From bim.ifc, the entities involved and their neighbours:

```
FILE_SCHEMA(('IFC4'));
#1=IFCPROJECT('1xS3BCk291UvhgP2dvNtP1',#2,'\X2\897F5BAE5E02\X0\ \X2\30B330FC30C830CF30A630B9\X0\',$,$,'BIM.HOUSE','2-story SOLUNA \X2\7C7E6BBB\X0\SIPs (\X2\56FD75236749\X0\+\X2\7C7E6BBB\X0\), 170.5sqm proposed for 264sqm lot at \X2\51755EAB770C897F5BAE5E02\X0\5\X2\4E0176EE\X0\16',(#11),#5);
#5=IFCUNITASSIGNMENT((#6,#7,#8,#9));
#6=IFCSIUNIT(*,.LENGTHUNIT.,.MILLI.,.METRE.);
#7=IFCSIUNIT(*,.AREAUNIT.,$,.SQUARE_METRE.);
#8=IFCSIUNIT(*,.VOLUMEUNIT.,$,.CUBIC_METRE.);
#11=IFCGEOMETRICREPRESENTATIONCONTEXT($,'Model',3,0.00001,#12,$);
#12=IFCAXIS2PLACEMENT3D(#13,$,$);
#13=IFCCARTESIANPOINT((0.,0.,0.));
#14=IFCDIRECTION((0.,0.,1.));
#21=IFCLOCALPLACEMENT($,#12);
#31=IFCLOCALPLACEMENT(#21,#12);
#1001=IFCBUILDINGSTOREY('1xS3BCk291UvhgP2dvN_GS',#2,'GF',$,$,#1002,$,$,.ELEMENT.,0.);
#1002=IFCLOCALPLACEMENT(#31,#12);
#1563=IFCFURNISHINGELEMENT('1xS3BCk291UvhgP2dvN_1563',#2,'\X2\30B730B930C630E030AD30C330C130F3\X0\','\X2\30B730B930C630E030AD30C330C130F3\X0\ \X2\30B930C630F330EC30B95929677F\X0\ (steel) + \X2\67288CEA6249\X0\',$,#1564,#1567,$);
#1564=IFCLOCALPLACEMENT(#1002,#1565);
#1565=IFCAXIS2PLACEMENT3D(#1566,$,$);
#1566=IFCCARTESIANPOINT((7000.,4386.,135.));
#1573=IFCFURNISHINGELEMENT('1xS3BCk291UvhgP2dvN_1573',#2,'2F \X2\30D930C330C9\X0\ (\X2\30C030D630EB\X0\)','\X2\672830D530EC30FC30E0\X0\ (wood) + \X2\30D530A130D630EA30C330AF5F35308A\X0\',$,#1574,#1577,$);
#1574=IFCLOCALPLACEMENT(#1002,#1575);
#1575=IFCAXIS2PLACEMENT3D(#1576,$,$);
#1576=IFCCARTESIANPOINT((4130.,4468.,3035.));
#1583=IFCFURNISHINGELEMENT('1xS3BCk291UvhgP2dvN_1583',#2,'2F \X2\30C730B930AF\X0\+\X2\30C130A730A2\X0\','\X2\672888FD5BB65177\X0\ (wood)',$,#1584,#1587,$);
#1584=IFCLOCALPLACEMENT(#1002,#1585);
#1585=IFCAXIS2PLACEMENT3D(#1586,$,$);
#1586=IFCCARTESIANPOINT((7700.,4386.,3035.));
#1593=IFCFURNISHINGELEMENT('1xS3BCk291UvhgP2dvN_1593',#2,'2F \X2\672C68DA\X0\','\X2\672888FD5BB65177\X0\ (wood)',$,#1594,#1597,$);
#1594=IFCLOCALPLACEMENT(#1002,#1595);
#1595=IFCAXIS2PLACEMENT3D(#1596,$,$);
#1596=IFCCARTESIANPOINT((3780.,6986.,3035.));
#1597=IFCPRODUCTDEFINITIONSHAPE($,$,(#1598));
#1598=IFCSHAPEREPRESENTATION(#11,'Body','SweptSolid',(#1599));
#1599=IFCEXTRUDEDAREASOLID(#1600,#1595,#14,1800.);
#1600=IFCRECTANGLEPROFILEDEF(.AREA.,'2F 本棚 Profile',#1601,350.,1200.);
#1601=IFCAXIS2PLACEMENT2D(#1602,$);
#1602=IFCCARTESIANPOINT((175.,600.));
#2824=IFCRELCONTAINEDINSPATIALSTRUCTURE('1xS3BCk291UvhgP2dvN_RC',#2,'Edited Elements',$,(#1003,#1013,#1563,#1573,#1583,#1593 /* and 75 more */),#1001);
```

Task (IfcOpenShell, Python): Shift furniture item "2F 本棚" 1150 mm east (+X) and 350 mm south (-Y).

```python
import ifcopenshell
import ifcopenshell.api.geometry
import ifcopenshell.util.placement
import ifcopenshell.util.unit

model = ifcopenshell.open("bim.ifc")
unit_scale = ifcopenshell.util.unit.calculate_unit_scale(model)

item = model.by_guid("1xS3BCk291UvhgP2dvN_1593")
matrix = ifcopenshell.util.placement.get_local_placement(item.ObjectPlacement)
matrix[0, 3] += 1.15 / unit_scale
matrix[1, 3] -= 0.35 / unit_scale
ifcopenshell.api.geometry.edit_object_placement(model, product=item, matrix=matrix, is_si=False)

print(ifcopenshell.util.placement.get_local_placement(item.ObjectPlacement).round(3) + 0.0)

model.write("bim_v2.ifc")
```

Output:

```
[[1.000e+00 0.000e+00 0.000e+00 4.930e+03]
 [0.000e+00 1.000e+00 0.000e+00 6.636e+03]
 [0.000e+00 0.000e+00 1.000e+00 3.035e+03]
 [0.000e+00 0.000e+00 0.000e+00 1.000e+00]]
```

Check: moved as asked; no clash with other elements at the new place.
